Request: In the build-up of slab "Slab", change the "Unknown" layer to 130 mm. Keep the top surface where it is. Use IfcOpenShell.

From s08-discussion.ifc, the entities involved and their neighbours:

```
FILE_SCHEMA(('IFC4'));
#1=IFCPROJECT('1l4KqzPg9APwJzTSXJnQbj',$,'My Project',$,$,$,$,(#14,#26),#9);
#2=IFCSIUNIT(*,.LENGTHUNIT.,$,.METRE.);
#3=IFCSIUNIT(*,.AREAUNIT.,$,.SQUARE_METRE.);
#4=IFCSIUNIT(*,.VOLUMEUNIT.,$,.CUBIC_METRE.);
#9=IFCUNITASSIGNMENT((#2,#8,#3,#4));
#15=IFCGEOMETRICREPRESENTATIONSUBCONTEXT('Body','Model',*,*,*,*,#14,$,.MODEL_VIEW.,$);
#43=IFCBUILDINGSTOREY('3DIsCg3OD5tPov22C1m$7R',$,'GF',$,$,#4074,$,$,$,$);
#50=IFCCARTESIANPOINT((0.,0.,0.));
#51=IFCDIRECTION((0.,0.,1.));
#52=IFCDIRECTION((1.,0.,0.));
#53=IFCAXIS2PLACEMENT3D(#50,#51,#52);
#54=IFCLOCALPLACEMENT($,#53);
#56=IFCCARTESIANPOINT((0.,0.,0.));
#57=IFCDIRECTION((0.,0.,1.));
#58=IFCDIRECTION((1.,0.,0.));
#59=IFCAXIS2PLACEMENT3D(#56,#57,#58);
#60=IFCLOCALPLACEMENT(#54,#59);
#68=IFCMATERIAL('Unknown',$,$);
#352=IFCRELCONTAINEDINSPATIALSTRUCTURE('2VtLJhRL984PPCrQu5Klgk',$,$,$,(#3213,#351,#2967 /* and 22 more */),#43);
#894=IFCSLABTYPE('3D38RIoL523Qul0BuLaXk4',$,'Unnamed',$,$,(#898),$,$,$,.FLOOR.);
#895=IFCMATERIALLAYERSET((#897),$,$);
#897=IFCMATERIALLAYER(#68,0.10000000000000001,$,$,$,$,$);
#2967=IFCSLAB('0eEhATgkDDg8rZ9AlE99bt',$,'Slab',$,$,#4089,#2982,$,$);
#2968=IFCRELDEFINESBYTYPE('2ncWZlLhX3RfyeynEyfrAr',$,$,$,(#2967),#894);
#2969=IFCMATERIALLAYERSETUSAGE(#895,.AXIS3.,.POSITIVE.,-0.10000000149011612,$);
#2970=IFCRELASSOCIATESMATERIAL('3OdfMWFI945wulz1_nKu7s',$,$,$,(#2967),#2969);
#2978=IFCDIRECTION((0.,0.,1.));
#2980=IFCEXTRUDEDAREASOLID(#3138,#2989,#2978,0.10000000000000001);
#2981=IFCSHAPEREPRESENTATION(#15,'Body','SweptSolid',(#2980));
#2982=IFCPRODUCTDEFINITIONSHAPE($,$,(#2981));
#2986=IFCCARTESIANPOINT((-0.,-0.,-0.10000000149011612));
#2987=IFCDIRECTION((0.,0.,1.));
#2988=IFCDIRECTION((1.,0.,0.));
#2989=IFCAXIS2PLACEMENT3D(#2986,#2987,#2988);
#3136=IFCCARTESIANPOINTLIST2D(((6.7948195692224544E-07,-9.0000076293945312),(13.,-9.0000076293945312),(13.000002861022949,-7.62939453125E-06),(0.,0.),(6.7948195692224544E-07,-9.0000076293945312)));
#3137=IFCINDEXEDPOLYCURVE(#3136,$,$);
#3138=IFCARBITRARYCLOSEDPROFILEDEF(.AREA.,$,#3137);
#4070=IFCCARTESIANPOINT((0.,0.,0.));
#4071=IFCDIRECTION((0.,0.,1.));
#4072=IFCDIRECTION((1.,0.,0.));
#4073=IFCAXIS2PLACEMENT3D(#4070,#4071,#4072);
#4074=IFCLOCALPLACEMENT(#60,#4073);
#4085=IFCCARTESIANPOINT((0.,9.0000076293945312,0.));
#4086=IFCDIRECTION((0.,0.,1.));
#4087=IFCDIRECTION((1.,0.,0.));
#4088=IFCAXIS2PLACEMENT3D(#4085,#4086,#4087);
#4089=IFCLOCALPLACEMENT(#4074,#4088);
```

```python
import ifcopenshell
import ifcopenshell.util.element
import ifcopenshell.util.representation

model = ifcopenshell.open("s08-discussion.ifc")

layer_set = model.by_id(895)
layer = next(l for l in layer_set.MaterialLayers if l.Material and l.Material.Name == "Unknown")
change = 0.13 - layer.LayerThickness
layer.LayerThickness += change

# Geometry does not follow the layer set by itself.
slabs = [e for e in ifcopenshell.util.element.get_elements_by_material(model, layer_set) if e.is_a("IfcSlab")]
for slab in sorted(slabs, key=lambda e: e.id()):
    body = ifcopenshell.util.representation.get_representation(slab, "Model", "Body")
    solid = body.Items[0]
    old_depth = solid.Depth
    solid.Depth += change
    # Extruded upwards: lower the start of the extrusion so the top stays.
    x, y, z = solid.Position.Location.Coordinates
    solid.Position.Location = model.createIfcCartesianPoint((x, y, z - change))
    print(slab.id(), f"{old_depth:g} -> {solid.Depth:g}")

# The layers are counted up from the underside, which has moved.
for usage in {ifcopenshell.util.element.get_material(slab) for slab in slabs}:
    usage.OffsetFromReferenceLine -= change

model.write("s08-discussion_updated.ifc")
```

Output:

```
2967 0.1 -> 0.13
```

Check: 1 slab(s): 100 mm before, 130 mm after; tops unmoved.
